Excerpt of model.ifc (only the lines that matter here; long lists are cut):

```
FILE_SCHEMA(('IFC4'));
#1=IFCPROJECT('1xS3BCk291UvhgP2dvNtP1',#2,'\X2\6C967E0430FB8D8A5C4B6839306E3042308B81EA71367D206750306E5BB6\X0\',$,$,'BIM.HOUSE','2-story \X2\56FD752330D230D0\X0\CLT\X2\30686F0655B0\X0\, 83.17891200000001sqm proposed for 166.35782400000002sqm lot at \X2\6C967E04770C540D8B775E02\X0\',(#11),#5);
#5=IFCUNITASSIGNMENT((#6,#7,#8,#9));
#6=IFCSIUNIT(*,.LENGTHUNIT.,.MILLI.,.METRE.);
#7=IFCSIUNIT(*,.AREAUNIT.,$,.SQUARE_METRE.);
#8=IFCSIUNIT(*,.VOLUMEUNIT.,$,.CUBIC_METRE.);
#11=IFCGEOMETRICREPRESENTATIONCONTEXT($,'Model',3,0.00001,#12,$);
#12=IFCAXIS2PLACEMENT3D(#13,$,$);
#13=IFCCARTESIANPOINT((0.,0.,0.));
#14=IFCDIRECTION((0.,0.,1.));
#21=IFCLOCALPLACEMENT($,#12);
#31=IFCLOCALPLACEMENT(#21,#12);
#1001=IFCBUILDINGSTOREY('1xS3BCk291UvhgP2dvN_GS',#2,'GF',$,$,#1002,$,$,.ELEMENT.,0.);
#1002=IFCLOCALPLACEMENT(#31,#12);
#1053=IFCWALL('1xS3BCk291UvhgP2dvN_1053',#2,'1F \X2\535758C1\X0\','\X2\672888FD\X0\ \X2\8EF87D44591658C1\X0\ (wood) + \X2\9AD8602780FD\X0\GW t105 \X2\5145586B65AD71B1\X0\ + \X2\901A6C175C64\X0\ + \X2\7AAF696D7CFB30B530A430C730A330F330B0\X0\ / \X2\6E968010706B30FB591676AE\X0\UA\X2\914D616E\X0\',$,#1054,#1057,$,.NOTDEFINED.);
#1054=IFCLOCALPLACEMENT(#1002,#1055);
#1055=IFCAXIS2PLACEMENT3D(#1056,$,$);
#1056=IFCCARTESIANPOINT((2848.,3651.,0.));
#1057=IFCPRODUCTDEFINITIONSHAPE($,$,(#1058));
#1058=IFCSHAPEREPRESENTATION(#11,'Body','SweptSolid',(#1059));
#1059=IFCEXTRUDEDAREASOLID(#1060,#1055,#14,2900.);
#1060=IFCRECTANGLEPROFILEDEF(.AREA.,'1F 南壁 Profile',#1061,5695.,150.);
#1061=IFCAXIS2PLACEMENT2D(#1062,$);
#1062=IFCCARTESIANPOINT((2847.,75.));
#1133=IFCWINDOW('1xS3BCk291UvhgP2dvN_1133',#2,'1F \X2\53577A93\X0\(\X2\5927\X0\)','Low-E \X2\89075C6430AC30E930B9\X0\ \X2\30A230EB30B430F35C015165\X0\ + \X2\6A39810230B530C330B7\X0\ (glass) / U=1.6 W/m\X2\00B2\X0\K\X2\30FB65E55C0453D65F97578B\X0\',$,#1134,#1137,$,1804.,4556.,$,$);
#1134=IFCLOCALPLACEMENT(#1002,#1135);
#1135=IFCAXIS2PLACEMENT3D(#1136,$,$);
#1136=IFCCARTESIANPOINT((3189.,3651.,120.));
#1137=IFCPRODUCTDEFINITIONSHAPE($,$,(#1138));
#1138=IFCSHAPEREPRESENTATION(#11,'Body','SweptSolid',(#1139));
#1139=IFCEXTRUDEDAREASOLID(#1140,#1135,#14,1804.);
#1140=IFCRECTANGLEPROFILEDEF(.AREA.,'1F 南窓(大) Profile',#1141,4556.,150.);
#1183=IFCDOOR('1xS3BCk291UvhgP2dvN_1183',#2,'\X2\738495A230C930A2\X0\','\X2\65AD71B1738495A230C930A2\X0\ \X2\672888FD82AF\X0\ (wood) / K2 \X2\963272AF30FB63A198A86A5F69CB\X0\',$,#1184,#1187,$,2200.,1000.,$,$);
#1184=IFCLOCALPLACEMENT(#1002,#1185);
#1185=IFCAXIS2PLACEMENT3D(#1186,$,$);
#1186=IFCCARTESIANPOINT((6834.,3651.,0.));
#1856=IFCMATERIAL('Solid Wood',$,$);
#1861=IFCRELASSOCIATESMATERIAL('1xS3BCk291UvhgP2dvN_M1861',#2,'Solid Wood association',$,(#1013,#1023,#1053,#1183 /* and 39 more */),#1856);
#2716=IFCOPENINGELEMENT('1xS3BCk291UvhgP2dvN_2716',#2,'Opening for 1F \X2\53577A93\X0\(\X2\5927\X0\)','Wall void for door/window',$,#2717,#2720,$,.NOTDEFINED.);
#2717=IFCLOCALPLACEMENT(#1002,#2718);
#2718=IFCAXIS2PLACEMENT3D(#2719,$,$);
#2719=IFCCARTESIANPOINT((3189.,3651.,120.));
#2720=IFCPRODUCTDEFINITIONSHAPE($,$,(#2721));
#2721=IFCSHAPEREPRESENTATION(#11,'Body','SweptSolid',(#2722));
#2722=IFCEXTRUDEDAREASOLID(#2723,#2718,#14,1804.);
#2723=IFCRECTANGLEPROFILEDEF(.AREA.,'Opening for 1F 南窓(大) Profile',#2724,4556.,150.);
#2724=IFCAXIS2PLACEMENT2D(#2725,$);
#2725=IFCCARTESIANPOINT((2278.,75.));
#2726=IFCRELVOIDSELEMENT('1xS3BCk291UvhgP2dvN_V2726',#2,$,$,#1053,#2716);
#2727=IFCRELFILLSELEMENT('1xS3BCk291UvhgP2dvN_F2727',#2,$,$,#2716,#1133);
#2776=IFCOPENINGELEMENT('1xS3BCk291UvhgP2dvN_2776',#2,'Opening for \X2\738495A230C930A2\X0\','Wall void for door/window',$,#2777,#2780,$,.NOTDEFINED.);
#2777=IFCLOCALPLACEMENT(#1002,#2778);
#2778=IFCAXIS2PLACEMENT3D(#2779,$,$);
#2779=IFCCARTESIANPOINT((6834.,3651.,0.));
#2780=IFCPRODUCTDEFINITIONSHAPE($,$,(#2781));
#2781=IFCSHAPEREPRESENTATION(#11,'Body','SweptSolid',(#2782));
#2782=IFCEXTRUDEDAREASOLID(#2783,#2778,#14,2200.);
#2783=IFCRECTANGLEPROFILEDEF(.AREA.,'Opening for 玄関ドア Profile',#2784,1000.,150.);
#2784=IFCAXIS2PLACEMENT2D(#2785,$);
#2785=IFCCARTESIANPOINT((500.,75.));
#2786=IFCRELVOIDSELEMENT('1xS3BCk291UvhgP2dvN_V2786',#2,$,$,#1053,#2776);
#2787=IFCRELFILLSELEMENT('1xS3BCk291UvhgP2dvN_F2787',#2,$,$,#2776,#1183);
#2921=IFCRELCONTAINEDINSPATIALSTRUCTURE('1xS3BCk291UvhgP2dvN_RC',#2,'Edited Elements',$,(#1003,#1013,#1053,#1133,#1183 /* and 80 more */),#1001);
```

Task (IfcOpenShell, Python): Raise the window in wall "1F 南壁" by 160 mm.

```python
import numpy as np
import ifcopenshell
import ifcopenshell.api.geometry
import ifcopenshell.util.placement
import ifcopenshell.util.unit

model = ifcopenshell.open("model.ifc")
unit_scale = ifcopenshell.util.unit.calculate_unit_scale(model)

window = model.by_guid("1xS3BCk291UvhgP2dvN_1133")
opening = window.FillsVoids[0].RelatingOpeningElement
dz = 0.16 / unit_scale

shift = np.array([0.0, 0.0, dz])
# The window is not placed relative to its opening, so move both.
for product in (opening, window):
    matrix = ifcopenshell.util.placement.get_local_placement(product.ObjectPlacement)
    matrix[:3, 3] += shift
    ifcopenshell.api.geometry.edit_object_placement(model, product=product, matrix=matrix, is_si=False)

print(f"moved by {dz * unit_scale:+.3f} m")

model.write("model_edited.ifc")
```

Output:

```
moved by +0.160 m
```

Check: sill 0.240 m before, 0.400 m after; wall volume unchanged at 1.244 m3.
